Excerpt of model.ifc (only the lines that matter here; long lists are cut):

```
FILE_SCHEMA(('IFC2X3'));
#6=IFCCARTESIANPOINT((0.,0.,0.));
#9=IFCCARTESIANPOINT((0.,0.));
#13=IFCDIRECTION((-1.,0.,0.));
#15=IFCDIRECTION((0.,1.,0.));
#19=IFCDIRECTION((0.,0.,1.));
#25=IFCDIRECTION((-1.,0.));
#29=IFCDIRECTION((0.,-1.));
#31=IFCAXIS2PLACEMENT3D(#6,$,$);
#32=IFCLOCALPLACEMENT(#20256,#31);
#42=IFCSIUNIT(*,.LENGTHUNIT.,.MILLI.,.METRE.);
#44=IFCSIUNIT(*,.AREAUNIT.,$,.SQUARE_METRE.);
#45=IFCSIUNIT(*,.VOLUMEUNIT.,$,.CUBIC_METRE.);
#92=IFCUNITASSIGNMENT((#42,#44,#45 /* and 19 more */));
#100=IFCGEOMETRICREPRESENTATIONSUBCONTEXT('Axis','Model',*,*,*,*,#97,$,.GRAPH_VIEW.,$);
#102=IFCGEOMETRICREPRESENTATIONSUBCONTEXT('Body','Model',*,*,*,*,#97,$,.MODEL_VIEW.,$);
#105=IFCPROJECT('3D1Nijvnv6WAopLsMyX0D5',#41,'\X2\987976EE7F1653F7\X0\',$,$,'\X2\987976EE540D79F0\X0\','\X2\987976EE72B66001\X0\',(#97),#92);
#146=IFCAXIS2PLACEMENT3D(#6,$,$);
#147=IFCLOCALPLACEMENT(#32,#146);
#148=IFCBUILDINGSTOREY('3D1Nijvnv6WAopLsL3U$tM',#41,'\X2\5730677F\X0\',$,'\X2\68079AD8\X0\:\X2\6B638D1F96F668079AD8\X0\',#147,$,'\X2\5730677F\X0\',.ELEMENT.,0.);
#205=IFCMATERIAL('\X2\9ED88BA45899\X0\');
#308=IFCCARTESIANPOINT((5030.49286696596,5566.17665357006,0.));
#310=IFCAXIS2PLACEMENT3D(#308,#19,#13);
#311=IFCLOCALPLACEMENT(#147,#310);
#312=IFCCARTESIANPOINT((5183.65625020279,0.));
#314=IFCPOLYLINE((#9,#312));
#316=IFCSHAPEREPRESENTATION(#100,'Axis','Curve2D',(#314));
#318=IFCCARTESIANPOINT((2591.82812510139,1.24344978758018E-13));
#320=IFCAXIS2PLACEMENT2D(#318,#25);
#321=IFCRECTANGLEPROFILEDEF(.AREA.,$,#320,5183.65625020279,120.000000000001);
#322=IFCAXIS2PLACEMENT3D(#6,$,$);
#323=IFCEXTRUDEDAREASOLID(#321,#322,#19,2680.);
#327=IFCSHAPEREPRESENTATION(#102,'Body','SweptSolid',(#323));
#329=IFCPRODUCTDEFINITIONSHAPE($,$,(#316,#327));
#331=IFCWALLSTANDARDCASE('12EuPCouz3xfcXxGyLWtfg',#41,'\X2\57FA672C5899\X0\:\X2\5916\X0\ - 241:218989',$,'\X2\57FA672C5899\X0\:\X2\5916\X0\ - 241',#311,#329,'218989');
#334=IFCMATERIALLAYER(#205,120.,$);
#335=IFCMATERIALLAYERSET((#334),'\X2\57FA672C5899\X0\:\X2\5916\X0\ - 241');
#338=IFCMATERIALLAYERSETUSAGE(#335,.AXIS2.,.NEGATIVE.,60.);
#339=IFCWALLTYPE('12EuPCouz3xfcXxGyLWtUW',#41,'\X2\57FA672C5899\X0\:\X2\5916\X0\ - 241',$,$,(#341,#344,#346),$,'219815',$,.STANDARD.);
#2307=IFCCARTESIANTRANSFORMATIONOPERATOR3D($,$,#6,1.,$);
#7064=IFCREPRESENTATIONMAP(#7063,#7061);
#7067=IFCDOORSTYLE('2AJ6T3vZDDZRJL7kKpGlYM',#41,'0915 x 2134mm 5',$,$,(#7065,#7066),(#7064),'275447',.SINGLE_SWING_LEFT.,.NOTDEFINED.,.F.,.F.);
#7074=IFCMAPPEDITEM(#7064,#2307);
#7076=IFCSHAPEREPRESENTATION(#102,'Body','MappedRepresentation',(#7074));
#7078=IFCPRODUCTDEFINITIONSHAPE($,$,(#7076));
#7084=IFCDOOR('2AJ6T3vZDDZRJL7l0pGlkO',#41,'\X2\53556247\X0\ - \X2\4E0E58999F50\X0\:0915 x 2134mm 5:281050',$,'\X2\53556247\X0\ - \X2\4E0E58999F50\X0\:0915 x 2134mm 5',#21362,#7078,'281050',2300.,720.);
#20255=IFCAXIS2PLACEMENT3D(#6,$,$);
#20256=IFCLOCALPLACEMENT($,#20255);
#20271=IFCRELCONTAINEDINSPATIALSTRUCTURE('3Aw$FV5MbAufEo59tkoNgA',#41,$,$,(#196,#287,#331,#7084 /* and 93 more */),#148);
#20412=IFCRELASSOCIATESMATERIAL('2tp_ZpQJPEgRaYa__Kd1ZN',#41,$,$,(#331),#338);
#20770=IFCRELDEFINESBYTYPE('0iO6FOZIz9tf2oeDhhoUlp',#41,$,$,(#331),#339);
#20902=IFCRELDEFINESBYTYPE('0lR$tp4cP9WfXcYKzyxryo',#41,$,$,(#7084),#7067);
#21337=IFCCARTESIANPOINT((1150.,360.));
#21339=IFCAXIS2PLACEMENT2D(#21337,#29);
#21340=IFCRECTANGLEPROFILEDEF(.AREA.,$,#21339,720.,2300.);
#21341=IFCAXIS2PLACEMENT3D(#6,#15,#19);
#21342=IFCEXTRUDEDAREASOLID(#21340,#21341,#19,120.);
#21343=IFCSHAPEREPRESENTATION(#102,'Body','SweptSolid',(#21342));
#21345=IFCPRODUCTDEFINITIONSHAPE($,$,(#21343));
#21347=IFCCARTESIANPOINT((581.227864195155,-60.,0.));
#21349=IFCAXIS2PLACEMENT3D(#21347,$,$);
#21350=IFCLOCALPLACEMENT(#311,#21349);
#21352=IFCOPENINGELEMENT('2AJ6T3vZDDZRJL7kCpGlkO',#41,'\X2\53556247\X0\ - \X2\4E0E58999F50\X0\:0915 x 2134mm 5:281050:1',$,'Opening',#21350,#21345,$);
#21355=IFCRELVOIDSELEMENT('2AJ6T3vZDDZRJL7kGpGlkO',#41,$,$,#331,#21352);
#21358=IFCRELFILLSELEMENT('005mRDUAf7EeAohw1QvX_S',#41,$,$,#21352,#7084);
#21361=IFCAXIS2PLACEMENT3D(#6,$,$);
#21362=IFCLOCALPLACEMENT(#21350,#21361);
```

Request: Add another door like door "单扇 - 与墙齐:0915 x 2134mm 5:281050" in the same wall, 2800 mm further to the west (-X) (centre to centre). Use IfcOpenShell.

```python
import ifcopenshell
import ifcopenshell.api.feature
import ifcopenshell.api.geometry
import ifcopenshell.api.root
import ifcopenshell.geom
import ifcopenshell.util.element
import ifcopenshell.util.placement
import ifcopenshell.util.shape
import ifcopenshell.util.unit

model = ifcopenshell.open("model.ifc")
unit_scale = ifcopenshell.util.unit.calculate_unit_scale(model)
settings = ifcopenshell.geom.settings()


def volume(element):
    """Net volume in cubic metres, openings subtracted."""
    shape = ifcopenshell.geom.create_shape(settings, element)
    return ifcopenshell.util.shape.get_volume(shape.geometry)


def reuse_history(source, copy):
    """copy_class also copies each property set's owner history, people and application; keep the originals."""
    for rel in copy.IsDefinedBy:
        if rel.is_a("IfcRelDefinesByProperties") and (history := rel.RelatingPropertyDefinition.OwnerHistory):
            rel.RelatingPropertyDefinition.OwnerHistory = source.OwnerHistory
            ifcopenshell.util.element.remove_deep2(model, history)


door = model.by_guid("2AJ6T3vZDDZRJL7l0pGlkO")
opening = door.FillsVoids[0].RelatingOpeningElement
wall = opening.VoidsElements[0].RelatingBuildingElement
before = volume(wall)
shift = ifcopenshell.util.placement.get_local_placement(wall.ObjectPlacement)[:3, 0] * 2.8 / unit_scale

# copy_class copies the void relationship, type, container and properties, but no geometry.
new_opening = ifcopenshell.api.root.copy_class(model, product=opening)
new_opening.Representation = ifcopenshell.util.element.copy_deep(
    model, opening.Representation, exclude=["IfcGeometricRepresentationContext", "IfcRepresentationMap"]
)
new_opening.Name = "单扇 - 与墙齐:0915 x 2134mm 5"
new_door = ifcopenshell.api.root.copy_class(model, product=door)
new_door.Representation = ifcopenshell.util.element.copy_deep(
    model, door.Representation, exclude=["IfcGeometricRepresentationContext", "IfcRepresentationMap"]
)
new_door.Name = "单扇 - 与墙齐:0915 x 2134mm 5"
new_door.Tag = None
reuse_history(door, new_door)
fills = ifcopenshell.api.feature.add_filling(model, opening=new_opening, element=new_door)
fills.OwnerHistory = new_door.OwnerHistory  # required in IFC2X3

for old, new in ((opening, new_opening), (door, new_door)):
    matrix = ifcopenshell.util.placement.get_local_placement(old.ObjectPlacement)
    matrix[:3, 3] += shift
    ifcopenshell.api.geometry.edit_object_placement(model, product=new, matrix=matrix, is_si=False)

after = volume(wall)

print(f"wall volume {before:.3f} -> {after:.3f} m3")

model.write("model_edited.ifc")
```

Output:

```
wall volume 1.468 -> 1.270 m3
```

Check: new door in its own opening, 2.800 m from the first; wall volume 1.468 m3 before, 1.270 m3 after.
